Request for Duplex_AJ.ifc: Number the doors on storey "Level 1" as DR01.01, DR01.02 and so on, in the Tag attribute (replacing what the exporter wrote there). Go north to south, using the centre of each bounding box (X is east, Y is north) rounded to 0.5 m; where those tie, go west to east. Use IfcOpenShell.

First a look at what the model holds.

```python
import ifcopenshell
import ifcopenshell.util.element
import ifcopenshell.util.placement

model = ifcopenshell.open("Duplex_AJ.ifc")
print(model.schema)
storey = next(s for s in model.by_type("IfcBuildingStorey") if s.Name == "Level 1")
doors = [e for e in ifcopenshell.util.element.get_decomposition(storey) if e.is_a("IfcDoor")]
for e in sorted(doors, key=lambda e: e.id()):
    origin = ifcopenshell.util.placement.get_local_placement(e.ObjectPlacement)[:3, 3]
    print(e.id(), e.Tag, e.Name, origin.round(2) + 0.0, sep=" | ")
```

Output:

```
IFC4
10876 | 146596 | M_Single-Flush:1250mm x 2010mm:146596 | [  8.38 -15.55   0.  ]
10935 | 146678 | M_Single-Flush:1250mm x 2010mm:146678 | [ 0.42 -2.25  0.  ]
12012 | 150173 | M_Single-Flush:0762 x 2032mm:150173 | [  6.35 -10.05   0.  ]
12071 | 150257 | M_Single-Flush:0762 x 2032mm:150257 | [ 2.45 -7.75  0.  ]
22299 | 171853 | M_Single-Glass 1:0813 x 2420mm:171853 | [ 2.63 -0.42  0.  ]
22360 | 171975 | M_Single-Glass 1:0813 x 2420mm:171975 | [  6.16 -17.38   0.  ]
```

```python
import ifcopenshell
import ifcopenshell.geom
import ifcopenshell.util.element
import ifcopenshell.util.shape

model = ifcopenshell.open("Duplex_AJ.ifc")
settings = ifcopenshell.geom.settings()
settings.set("use-world-coords", True)


def centre(element):
    shape = ifcopenshell.geom.create_shape(settings, element)
    return ifcopenshell.util.shape.get_bbox_centroid(shape.geometry)


storey = next(s for s in model.by_type("IfcBuildingStorey") if s.Name == "Level 1")
doors = [e for e in ifcopenshell.util.element.get_decomposition(storey) if e.is_a("IfcDoor")]

# Insertion points can sit at a corner or the storey origin, so sort by the geometry (in metres).
centres = {e: centre(e) for e in doors}
doors.sort(key=lambda e: (-round(centres[e][1] / 0.5), centres[e][0]))

for i, e in enumerate(doors, start=1):
    number = f"DR01.{i:02d}"
    e.Tag = number
    print(e.id(), number)

model.write("Duplex_AJ_updated.ifc")
```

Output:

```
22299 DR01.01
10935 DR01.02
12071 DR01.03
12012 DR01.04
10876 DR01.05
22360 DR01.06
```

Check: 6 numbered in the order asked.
